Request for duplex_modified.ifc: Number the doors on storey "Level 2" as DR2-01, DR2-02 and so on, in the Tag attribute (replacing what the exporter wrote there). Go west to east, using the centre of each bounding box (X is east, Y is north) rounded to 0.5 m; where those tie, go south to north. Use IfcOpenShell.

First a look at what the model holds.

```python
import ifcopenshell
import ifcopenshell.util.element
import ifcopenshell.util.placement

model = ifcopenshell.open("duplex_modified.ifc")
print(model.schema)
storey = next(s for s in model.by_type("IfcBuildingStorey") if s.Name == "Level 2")
doors = [e for e in ifcopenshell.util.element.get_decomposition(storey) if e.is_a("IfcDoor")]
for e in sorted(doors, key=lambda e: e.id()):
    origin = ifcopenshell.util.placement.get_local_placement(e.ObjectPlacement)[:3, 3]
    print(e.id(), e.Tag, e.Name, origin.round(2) + 0.0, sep=" | ")
```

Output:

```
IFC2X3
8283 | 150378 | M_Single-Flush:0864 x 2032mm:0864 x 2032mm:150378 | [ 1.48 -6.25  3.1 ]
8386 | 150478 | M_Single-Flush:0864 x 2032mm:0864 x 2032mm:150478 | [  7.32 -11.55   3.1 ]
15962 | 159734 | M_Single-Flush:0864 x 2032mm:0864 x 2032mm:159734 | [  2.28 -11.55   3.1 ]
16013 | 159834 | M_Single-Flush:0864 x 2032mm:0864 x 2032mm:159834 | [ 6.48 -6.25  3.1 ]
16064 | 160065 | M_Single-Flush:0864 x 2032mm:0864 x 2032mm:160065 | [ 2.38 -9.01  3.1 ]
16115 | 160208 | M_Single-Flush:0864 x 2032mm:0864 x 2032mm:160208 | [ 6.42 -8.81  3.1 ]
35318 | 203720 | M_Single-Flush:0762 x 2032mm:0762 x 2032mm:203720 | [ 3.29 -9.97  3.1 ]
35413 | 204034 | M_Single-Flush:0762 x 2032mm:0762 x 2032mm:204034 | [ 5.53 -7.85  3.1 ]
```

```python
import ifcopenshell
import ifcopenshell.geom
import ifcopenshell.util.element
import ifcopenshell.util.shape

model = ifcopenshell.open("duplex_modified.ifc")
settings = ifcopenshell.geom.settings()
settings.set("use-world-coords", True)


def centre(element):
    shape = ifcopenshell.geom.create_shape(settings, element)
    return ifcopenshell.util.shape.get_bbox_centroid(shape.geometry)


storey = next(s for s in model.by_type("IfcBuildingStorey") if s.Name == "Level 2")
doors = [e for e in ifcopenshell.util.element.get_decomposition(storey) if e.is_a("IfcDoor")]

# Insertion points can sit at a corner or the storey origin, so sort by the geometry (in metres).
centres = {e: centre(e) for e in doors}
doors.sort(key=lambda e: (round(centres[e][0] / 0.5), centres[e][1]))

for i, e in enumerate(doors, start=1):
    number = f"DR2-{i:02d}"
    e.Tag = number
    print(e.id(), number)

model.write("duplex_modified-out.ifc")
```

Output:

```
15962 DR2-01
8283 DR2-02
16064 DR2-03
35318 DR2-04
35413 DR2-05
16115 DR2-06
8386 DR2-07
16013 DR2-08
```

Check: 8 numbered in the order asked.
